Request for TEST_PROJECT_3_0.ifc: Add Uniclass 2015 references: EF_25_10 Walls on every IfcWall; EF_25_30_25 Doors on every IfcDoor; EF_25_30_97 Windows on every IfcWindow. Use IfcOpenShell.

First a look at what the model holds.

```python
import ifcopenshell

model = ifcopenshell.open("TEST_PROJECT_3_0.ifc")
print(model.schema)
print("classifications:", [c.Name for c in model.by_type("IfcClassification")])
for ifc_class in ("IfcDoor", "IfcRoof", "IfcStair", "IfcWall", "IfcWindow"):
    print(ifc_class, len(model.by_type(ifc_class)))
```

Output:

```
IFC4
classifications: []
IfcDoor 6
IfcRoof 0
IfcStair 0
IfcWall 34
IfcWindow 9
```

```python
import ifcopenshell
import ifcopenshell.api.classification

model = ifcopenshell.open("TEST_PROJECT_3_0.ifc")

system = ifcopenshell.api.classification.add_classification(model, classification="Uniclass 2015")

codes = {
    "IfcWall": ("EF_25_10", "Walls"),
    "IfcDoor": ("EF_25_30_25", "Doors"),
    "IfcWindow": ("EF_25_30_97", "Windows"),
}
for ifc_class, (code, name) in codes.items():
    products = model.by_type(ifc_class)
    ifcopenshell.api.classification.add_reference(
        model, products=products, classification=system, identification=code, name=name
    )
    print(code, len(products))

model.write("TEST_PROJECT_3_0_v2.ifc")
```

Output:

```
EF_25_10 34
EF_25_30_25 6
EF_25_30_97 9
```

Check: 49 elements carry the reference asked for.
